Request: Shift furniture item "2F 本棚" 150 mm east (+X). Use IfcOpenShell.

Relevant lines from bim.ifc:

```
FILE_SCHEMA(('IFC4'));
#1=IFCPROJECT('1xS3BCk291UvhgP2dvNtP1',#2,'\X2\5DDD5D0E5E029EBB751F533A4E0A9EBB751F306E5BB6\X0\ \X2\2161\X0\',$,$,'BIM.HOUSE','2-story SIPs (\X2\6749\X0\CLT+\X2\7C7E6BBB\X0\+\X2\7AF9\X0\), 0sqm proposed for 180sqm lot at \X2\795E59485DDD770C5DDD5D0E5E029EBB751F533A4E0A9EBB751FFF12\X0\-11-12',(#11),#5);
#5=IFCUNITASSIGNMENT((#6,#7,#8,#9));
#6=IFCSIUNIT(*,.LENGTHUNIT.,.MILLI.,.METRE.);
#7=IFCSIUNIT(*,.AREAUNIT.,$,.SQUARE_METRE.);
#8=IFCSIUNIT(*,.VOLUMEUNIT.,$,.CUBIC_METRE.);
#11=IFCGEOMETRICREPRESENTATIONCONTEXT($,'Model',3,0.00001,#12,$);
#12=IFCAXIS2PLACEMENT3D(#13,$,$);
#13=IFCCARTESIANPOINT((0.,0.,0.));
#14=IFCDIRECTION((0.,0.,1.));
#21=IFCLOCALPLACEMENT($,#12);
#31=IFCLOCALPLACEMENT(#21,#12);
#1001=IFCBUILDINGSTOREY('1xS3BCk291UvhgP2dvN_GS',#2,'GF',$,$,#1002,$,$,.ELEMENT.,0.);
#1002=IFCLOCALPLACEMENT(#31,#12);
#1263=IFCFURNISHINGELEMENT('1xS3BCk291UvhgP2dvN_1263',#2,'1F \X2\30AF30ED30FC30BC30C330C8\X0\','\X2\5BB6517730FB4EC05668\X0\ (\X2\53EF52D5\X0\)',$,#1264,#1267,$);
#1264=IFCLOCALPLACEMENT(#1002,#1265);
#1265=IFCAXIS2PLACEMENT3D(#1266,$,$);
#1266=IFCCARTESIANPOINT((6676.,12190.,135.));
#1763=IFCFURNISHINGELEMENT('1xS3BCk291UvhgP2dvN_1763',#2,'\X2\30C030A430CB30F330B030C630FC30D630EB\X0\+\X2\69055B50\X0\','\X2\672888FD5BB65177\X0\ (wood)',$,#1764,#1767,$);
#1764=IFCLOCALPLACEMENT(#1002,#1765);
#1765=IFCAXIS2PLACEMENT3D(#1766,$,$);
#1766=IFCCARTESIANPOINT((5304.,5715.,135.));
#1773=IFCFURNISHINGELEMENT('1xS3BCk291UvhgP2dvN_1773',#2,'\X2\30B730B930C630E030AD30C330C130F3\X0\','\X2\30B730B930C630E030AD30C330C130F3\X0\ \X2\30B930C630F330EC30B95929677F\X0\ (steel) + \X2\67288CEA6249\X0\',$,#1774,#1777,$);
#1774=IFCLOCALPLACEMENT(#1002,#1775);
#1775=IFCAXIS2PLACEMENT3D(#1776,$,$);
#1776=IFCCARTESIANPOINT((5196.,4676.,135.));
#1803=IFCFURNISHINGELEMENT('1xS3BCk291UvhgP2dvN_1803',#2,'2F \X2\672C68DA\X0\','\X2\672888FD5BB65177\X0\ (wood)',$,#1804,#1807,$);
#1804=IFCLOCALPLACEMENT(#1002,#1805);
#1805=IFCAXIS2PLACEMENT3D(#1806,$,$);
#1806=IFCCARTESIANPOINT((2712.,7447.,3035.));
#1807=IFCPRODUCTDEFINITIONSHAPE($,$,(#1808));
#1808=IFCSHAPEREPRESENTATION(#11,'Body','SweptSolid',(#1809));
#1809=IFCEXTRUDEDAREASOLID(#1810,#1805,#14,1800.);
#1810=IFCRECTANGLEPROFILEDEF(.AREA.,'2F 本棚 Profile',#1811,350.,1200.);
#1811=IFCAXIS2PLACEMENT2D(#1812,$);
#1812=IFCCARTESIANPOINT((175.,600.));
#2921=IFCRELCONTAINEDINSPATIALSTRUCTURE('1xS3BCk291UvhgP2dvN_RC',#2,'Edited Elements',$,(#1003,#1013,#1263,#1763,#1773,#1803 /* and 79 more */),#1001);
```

```python
import ifcopenshell
import ifcopenshell.api.geometry
import ifcopenshell.util.placement
import ifcopenshell.util.unit

model = ifcopenshell.open("bim.ifc")
unit_scale = ifcopenshell.util.unit.calculate_unit_scale(model)

item = model.by_guid("1xS3BCk291UvhgP2dvN_1803")
matrix = ifcopenshell.util.placement.get_local_placement(item.ObjectPlacement)
matrix[0, 3] += 0.15 / unit_scale
ifcopenshell.api.geometry.edit_object_placement(model, product=item, matrix=matrix, is_si=False)

print(ifcopenshell.util.placement.get_local_placement(item.ObjectPlacement).round(3) + 0.0)

model.write("bim_edited.ifc")
```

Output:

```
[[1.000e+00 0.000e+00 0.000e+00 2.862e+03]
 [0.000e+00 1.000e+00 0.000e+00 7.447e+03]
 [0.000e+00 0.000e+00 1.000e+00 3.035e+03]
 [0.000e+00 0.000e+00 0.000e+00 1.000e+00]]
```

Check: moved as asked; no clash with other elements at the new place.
